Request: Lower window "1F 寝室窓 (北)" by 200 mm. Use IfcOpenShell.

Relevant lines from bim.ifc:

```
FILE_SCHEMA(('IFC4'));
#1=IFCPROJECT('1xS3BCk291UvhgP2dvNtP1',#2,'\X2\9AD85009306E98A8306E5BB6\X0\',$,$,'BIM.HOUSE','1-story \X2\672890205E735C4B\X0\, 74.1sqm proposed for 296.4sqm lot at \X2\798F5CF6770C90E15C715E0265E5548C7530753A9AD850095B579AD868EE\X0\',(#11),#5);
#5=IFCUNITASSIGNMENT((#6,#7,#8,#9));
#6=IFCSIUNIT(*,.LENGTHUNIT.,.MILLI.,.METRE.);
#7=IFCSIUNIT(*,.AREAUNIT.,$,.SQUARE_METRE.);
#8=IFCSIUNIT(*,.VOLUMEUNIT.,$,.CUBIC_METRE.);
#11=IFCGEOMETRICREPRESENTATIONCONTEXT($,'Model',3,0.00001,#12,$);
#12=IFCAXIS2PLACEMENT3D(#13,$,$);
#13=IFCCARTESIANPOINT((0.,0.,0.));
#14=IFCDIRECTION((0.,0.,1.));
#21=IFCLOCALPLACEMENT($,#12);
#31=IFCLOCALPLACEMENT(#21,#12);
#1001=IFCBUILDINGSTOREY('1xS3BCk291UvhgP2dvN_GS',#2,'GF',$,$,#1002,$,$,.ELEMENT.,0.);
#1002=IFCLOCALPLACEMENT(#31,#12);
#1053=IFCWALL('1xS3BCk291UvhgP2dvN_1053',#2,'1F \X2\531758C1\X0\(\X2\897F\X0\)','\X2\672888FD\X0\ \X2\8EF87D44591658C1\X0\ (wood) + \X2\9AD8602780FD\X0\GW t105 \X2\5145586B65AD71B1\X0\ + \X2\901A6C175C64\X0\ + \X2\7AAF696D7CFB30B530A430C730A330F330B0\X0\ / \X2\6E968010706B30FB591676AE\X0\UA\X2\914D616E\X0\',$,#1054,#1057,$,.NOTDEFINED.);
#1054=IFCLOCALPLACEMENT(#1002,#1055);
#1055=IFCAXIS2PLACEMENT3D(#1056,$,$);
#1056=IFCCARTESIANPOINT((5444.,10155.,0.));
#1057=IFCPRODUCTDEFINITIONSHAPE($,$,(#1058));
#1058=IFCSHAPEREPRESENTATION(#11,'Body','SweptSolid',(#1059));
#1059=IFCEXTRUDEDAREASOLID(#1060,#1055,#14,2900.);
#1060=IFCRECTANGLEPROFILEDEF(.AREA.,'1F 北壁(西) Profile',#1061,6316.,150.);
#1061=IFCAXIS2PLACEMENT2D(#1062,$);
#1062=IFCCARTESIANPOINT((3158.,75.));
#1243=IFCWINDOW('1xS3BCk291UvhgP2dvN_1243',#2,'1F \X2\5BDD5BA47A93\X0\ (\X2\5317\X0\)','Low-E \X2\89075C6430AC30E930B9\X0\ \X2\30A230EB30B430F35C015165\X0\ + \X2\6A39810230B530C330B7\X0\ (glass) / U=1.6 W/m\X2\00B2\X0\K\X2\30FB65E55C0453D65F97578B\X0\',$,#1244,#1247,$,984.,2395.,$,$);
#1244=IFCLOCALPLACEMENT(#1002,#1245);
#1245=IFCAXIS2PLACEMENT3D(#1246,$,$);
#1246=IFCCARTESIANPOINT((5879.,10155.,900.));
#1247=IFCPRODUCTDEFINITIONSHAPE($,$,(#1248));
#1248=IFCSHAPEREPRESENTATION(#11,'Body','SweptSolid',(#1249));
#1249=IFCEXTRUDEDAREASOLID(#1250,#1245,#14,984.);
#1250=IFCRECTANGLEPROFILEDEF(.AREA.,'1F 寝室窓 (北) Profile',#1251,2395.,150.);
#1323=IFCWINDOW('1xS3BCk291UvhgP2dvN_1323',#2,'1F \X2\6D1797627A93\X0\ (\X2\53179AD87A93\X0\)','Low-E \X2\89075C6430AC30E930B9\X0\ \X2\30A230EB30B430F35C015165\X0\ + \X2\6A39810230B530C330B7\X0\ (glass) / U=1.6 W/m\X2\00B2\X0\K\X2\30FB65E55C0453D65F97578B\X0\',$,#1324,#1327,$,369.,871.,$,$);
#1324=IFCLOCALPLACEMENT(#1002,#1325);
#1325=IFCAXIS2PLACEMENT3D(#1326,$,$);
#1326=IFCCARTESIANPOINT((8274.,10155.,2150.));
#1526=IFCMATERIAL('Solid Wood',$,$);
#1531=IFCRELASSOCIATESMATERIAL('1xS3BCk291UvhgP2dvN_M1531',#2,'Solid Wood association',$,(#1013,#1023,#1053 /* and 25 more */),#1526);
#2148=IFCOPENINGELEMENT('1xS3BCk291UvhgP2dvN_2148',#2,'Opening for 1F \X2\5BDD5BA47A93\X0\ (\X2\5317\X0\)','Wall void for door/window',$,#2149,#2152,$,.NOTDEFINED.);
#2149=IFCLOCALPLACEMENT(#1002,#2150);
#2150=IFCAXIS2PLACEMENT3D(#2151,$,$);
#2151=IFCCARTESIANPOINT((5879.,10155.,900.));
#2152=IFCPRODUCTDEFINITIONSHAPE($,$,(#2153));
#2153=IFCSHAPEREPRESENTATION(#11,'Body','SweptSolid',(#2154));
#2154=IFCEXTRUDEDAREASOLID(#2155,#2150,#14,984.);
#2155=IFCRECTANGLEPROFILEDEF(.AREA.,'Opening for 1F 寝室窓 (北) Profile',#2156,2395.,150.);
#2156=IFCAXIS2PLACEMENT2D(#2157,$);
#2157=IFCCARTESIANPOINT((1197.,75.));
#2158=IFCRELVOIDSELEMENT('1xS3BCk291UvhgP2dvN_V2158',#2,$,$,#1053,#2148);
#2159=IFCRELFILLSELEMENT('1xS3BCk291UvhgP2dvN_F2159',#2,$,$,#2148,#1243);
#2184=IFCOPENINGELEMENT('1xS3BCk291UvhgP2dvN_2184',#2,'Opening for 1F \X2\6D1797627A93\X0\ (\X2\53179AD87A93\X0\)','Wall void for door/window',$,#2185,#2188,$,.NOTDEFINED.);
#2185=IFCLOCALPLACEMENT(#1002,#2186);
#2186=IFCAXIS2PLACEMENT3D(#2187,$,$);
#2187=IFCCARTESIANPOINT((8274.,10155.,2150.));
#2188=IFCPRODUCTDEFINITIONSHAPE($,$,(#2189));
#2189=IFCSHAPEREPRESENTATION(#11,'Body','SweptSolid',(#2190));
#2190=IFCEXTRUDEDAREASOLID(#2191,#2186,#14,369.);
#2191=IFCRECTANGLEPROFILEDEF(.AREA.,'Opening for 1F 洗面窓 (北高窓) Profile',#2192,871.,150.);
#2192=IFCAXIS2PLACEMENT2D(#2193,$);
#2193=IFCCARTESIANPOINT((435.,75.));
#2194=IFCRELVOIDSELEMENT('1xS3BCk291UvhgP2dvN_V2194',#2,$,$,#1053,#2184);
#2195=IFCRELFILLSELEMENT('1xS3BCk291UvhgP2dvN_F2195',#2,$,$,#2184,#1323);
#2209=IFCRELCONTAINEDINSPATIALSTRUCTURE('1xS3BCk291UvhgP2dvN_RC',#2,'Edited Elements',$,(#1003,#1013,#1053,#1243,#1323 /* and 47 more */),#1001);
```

```python
import numpy as np
import ifcopenshell
import ifcopenshell.api.geometry
import ifcopenshell.util.placement
import ifcopenshell.util.unit

model = ifcopenshell.open("bim.ifc")
unit_scale = ifcopenshell.util.unit.calculate_unit_scale(model)

window = model.by_guid("1xS3BCk291UvhgP2dvN_1243")
opening = window.FillsVoids[0].RelatingOpeningElement
dz = -200.0

shift = np.array([0.0, 0.0, dz])
# The window is not placed relative to its opening, so move both.
for product in (opening, window):
    matrix = ifcopenshell.util.placement.get_local_placement(product.ObjectPlacement)
    matrix[:3, 3] += shift
    ifcopenshell.api.geometry.edit_object_placement(model, product=product, matrix=matrix, is_si=False)

print(f"moved by {dz * unit_scale:+.3f} m")

model.write("bim-out.ifc")
```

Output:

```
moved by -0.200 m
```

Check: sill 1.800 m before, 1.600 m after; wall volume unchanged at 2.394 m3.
